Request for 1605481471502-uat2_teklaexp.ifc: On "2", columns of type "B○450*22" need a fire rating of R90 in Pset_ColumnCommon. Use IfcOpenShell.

First a look at what the model holds.

```python
import ifcopenshell
import ifcopenshell.util.element

model = ifcopenshell.open("1605481471502-uat2_teklaexp.ifc")
print(model.schema)
storey = next(s for s in model.by_type("IfcBuildingStorey") if s.Name == "2")
columns = [e for e in ifcopenshell.util.element.get_decomposition(storey) if e.is_a("IfcColumn")]
seen = {}
for e in columns:
    element_type = ifcopenshell.util.element.get_type(e)
    key = (element_type.Name if element_type != e and element_type else None, ifcopenshell.util.element.get_pset(e, "Pset_ColumnCommon", "FireRating"))
    seen[key] = seen.get(key, 0) + 1
for (name, value), count in sorted(seen.items(), key=str):
    print(count, "x", name, "|", value)
```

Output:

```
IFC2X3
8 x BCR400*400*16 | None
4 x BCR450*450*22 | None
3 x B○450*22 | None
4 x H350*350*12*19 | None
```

```python
import ifcopenshell
import ifcopenshell.api.pset
import ifcopenshell.util.element

model = ifcopenshell.open("1605481471502-uat2_teklaexp.ifc")

storey = next(s for s in model.by_type("IfcBuildingStorey") if s.Name == "2")
columns = [e for e in ifcopenshell.util.element.get_decomposition(storey) if e.is_a("IfcColumn")]

count = 0
for e in columns:
    element_type = ifcopenshell.util.element.get_type(e)
    if element_type in (None, e) or element_type.Name != "B○450*22":
        continue
    found = ifcopenshell.util.element.get_pset(e, "Pset_ColumnCommon", should_inherit=False)
    if found:
        pset = model.by_id(found["id"])
        if len(ifcopenshell.util.element.get_elements_by_pset(pset)) > 1:
            pset = ifcopenshell.api.pset.unshare_pset(model, products=[e], pset=pset)[0]
    else:
        pset = ifcopenshell.api.pset.add_pset(model, product=e, name="Pset_ColumnCommon")
    ifcopenshell.api.pset.edit_pset(model, pset=pset, properties={"FireRating": "R90"})
    count += 1

print(count, "columns updated")

model.write("1605481471502-uat2_teklaexp_updated.ifc")
```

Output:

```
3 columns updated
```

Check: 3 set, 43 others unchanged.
